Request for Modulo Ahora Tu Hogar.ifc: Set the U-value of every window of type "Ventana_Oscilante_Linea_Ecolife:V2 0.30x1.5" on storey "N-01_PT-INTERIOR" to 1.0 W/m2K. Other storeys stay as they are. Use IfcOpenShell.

First a look at what the model holds.

```python
import ifcopenshell
import ifcopenshell.util.element

model = ifcopenshell.open("Modulo Ahora Tu Hogar.ifc")
print(model.schema)
storey = next(s for s in model.by_type("IfcBuildingStorey") if s.Name == "N-01_PT-INTERIOR")
windows = [e for e in ifcopenshell.util.element.get_decomposition(storey) if e.is_a("IfcWindow")]
seen = {}
for e in windows:
    element_type = ifcopenshell.util.element.get_type(e)
    key = (element_type.Name if element_type != e and element_type else None, ifcopenshell.util.element.get_pset(e, "Pset_WindowCommon", "ThermalTransmittance"))
    seen[key] = seen.get(key, 0) + 1
for (name, value), count in sorted(seen.items(), key=str):
    print(count, "x", name, "|", value)
```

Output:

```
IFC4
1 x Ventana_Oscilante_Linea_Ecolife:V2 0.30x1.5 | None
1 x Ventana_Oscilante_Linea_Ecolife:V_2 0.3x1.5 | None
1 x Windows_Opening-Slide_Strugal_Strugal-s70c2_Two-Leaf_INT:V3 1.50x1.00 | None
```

```python
import ifcopenshell
import ifcopenshell.api.pset
import ifcopenshell.util.element

model = ifcopenshell.open("Modulo Ahora Tu Hogar.ifc")

storey = next(s for s in model.by_type("IfcBuildingStorey") if s.Name == "N-01_PT-INTERIOR")
windows = [e for e in ifcopenshell.util.element.get_decomposition(storey) if e.is_a("IfcWindow")]

count = 0
for e in windows:
    element_type = ifcopenshell.util.element.get_type(e)
    if element_type in (None, e) or element_type.Name != "Ventana_Oscilante_Linea_Ecolife:V2 0.30x1.5":
        continue
    # add_pset returns the element's existing set when there is one.
    pset = ifcopenshell.api.pset.add_pset(model, product=e, name="Pset_WindowCommon")
    ifcopenshell.api.pset.edit_pset(model, pset=pset, properties={"ThermalTransmittance": 1.0})
    count += 1

print(count, "windows updated")

model.write("Modulo Ahora Tu Hogar_rev.ifc")
```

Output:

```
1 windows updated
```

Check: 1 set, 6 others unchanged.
